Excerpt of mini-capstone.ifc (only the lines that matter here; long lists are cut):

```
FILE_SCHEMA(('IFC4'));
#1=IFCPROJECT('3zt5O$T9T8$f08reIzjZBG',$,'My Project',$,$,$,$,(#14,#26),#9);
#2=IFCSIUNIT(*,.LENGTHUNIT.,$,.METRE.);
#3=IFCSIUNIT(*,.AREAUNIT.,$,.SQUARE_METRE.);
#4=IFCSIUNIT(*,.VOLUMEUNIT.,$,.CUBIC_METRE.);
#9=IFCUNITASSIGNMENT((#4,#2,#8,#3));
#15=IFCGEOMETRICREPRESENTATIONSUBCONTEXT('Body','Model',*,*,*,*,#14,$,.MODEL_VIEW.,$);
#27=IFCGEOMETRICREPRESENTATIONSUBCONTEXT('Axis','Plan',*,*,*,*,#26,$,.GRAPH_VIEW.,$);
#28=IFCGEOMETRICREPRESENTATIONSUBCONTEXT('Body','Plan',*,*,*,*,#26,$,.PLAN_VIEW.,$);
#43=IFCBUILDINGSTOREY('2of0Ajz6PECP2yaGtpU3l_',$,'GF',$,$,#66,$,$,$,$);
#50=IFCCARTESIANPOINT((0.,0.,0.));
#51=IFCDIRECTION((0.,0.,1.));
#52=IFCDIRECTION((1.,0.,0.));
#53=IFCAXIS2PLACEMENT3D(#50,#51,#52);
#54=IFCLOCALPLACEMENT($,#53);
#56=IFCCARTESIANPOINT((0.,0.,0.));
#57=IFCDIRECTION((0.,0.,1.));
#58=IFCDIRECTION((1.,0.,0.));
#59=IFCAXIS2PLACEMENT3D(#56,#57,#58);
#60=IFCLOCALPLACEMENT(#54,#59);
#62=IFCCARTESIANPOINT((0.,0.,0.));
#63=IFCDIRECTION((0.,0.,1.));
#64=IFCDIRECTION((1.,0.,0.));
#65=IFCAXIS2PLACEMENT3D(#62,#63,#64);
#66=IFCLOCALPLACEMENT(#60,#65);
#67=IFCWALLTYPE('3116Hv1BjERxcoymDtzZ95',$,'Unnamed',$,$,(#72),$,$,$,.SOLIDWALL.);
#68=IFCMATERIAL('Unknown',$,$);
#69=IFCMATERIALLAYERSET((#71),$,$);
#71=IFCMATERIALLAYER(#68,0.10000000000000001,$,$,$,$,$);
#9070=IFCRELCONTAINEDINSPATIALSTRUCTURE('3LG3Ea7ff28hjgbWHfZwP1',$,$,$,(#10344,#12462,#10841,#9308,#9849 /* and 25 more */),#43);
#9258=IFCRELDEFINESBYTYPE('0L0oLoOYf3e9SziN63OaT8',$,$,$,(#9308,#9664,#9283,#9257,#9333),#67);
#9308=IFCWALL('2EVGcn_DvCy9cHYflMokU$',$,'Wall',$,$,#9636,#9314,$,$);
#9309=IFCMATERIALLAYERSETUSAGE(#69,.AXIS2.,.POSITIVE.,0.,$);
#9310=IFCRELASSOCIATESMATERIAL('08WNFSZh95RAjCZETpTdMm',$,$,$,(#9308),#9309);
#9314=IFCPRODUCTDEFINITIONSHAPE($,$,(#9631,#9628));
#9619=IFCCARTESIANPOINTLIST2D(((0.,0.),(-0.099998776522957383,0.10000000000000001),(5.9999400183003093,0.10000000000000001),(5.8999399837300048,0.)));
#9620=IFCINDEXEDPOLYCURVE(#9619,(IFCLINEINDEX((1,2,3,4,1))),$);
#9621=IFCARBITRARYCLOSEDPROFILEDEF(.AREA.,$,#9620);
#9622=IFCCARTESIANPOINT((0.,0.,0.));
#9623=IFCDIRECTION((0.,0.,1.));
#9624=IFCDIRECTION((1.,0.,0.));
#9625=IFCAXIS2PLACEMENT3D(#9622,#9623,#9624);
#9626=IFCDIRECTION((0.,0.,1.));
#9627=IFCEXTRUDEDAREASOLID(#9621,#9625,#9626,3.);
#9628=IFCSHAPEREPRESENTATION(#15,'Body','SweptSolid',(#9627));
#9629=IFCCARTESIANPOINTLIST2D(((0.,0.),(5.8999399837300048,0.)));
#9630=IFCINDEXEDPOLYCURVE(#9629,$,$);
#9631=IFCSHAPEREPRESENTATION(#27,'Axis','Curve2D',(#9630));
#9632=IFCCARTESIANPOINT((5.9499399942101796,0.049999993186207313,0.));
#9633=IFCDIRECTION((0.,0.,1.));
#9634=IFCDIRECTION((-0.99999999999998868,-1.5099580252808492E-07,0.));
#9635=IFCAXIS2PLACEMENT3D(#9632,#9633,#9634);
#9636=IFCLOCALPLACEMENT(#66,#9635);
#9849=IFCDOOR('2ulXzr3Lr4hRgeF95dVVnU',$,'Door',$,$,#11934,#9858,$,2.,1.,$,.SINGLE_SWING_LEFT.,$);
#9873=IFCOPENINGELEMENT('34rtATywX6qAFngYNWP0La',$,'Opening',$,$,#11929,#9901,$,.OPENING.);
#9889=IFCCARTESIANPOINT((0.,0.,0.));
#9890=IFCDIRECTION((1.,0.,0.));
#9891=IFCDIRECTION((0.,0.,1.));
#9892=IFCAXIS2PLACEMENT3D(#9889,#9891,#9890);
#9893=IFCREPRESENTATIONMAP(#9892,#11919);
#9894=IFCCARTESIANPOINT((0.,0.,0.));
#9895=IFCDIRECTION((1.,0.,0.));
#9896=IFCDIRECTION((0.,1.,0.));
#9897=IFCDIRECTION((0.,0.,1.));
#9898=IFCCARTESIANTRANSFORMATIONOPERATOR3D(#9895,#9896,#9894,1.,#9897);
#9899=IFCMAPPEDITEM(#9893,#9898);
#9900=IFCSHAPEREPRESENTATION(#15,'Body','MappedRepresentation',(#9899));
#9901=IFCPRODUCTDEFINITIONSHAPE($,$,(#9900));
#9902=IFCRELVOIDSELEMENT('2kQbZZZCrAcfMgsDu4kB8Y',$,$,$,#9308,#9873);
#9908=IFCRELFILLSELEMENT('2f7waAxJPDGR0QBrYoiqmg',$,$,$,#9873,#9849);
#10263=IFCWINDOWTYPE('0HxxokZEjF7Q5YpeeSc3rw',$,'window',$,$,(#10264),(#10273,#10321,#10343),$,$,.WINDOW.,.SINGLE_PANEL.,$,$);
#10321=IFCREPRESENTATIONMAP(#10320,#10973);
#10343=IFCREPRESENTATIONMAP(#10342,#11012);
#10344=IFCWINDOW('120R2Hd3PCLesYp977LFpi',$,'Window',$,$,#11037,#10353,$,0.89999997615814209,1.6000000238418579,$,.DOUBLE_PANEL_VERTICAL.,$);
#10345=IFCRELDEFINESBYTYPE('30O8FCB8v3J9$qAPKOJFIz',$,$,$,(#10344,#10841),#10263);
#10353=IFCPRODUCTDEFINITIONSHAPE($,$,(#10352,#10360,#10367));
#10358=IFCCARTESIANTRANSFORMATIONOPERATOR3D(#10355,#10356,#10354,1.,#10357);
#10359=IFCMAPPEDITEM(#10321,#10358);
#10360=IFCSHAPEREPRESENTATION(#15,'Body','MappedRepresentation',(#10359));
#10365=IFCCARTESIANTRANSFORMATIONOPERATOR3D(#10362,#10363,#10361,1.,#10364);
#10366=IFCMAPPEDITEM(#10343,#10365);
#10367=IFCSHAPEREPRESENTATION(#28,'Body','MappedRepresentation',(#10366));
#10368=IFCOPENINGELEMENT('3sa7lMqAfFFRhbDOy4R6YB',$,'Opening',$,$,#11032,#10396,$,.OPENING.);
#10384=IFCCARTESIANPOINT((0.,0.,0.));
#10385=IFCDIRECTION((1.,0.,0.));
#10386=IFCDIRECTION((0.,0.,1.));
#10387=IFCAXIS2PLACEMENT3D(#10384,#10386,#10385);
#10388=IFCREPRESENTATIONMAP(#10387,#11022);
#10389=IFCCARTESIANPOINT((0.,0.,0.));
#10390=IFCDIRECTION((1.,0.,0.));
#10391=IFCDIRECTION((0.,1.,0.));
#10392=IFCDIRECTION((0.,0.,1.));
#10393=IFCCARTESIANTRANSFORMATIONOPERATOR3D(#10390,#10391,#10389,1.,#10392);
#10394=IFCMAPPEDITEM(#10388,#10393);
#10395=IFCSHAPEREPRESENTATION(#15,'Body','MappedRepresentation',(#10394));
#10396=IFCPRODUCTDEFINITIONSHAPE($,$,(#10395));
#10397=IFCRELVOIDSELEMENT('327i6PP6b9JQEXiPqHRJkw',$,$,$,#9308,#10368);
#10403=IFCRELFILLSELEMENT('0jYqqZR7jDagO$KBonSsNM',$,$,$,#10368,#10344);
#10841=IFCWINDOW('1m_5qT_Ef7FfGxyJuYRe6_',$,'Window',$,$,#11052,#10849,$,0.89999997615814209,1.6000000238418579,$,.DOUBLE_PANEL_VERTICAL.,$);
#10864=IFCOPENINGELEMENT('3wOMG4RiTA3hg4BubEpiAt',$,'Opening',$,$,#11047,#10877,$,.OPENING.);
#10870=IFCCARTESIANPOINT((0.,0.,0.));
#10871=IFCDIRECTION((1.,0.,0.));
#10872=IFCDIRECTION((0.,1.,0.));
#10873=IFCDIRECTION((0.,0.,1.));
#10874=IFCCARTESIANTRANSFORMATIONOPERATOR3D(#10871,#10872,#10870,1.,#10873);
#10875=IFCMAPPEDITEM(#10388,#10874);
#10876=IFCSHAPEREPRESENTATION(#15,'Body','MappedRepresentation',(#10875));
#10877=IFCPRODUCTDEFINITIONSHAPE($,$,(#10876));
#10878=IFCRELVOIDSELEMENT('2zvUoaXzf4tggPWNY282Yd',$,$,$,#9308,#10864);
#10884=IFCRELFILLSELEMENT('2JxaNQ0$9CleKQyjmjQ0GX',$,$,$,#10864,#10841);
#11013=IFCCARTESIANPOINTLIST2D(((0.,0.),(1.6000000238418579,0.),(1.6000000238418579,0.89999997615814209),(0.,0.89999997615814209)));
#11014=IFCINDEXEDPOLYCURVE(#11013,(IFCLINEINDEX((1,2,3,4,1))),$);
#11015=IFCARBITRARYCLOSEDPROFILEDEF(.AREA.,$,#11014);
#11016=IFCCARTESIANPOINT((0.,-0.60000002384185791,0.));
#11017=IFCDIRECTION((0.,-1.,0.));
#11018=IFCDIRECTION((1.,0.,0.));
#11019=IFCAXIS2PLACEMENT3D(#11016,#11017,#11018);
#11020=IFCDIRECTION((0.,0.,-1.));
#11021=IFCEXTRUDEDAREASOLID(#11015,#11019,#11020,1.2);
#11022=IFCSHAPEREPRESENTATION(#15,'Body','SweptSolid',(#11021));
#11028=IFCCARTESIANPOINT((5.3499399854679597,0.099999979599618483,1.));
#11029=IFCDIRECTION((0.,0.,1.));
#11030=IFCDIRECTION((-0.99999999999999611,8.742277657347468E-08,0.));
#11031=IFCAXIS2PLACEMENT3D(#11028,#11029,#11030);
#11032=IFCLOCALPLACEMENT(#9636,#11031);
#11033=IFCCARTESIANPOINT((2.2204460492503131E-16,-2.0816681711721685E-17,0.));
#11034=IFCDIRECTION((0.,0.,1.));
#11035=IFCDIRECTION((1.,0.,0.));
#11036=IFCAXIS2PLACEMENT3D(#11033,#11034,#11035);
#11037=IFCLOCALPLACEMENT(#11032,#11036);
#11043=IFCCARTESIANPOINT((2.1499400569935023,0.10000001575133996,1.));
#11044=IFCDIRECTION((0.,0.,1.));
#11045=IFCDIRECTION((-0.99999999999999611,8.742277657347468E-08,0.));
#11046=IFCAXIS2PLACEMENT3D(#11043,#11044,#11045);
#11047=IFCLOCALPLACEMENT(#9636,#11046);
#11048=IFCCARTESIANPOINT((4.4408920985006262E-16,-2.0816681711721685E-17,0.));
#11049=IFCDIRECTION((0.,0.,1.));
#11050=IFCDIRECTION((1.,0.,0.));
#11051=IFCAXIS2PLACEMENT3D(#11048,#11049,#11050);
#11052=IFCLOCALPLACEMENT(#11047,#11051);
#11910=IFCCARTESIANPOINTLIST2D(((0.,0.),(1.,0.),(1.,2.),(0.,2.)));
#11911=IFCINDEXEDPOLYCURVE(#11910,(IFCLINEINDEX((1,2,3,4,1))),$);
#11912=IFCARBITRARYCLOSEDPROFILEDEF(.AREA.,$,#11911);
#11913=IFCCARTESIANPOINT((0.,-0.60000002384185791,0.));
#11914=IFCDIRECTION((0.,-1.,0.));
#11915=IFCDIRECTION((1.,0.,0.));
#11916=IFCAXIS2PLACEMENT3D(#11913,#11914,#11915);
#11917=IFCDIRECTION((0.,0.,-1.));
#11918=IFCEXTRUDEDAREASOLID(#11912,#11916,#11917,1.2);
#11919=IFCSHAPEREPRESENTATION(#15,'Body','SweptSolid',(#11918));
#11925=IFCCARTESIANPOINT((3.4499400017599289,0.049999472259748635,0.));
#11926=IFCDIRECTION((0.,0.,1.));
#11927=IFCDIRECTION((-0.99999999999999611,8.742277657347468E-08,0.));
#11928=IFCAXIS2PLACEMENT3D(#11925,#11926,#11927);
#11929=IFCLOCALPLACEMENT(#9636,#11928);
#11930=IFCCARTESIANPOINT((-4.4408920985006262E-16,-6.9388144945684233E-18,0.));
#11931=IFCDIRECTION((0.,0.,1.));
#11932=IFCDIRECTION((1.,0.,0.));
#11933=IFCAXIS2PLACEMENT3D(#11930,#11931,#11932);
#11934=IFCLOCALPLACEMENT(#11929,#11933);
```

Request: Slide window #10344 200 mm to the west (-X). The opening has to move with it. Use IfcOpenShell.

```python
import ifcopenshell
import ifcopenshell.api.geometry
import ifcopenshell.util.placement
import ifcopenshell.util.unit

model = ifcopenshell.open("mini-capstone.ifc")
unit_scale = ifcopenshell.util.unit.calculate_unit_scale(model)

window = model.by_guid("120R2Hd3PCLesYp977LFpi")
opening = window.FillsVoids[0].RelatingOpeningElement
wall = opening.VoidsElements[0].RelatingBuildingElement

wall_matrix = ifcopenshell.util.placement.get_local_placement(wall.ObjectPlacement)
shift = wall_matrix[:3, 0] * 0.2 / unit_scale
before = ifcopenshell.util.placement.get_local_placement(window.ObjectPlacement)[:3, 3].copy()

# The window is placed relative to its opening, so it follows when the opening moves.
matrix = ifcopenshell.util.placement.get_local_placement(opening.ObjectPlacement)
matrix[:3, 3] += shift
ifcopenshell.api.geometry.edit_object_placement(
    model, product=opening, matrix=matrix, is_si=False, should_transform_children=True
)

after = ifcopenshell.util.placement.get_local_placement(window.ObjectPlacement)[:3, 3]
print("window moved by", (after - before).round(3) + 0.0)

model.write("mini-capstone_edited.ifc")
```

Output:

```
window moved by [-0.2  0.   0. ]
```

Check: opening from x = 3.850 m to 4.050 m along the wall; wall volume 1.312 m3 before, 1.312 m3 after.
